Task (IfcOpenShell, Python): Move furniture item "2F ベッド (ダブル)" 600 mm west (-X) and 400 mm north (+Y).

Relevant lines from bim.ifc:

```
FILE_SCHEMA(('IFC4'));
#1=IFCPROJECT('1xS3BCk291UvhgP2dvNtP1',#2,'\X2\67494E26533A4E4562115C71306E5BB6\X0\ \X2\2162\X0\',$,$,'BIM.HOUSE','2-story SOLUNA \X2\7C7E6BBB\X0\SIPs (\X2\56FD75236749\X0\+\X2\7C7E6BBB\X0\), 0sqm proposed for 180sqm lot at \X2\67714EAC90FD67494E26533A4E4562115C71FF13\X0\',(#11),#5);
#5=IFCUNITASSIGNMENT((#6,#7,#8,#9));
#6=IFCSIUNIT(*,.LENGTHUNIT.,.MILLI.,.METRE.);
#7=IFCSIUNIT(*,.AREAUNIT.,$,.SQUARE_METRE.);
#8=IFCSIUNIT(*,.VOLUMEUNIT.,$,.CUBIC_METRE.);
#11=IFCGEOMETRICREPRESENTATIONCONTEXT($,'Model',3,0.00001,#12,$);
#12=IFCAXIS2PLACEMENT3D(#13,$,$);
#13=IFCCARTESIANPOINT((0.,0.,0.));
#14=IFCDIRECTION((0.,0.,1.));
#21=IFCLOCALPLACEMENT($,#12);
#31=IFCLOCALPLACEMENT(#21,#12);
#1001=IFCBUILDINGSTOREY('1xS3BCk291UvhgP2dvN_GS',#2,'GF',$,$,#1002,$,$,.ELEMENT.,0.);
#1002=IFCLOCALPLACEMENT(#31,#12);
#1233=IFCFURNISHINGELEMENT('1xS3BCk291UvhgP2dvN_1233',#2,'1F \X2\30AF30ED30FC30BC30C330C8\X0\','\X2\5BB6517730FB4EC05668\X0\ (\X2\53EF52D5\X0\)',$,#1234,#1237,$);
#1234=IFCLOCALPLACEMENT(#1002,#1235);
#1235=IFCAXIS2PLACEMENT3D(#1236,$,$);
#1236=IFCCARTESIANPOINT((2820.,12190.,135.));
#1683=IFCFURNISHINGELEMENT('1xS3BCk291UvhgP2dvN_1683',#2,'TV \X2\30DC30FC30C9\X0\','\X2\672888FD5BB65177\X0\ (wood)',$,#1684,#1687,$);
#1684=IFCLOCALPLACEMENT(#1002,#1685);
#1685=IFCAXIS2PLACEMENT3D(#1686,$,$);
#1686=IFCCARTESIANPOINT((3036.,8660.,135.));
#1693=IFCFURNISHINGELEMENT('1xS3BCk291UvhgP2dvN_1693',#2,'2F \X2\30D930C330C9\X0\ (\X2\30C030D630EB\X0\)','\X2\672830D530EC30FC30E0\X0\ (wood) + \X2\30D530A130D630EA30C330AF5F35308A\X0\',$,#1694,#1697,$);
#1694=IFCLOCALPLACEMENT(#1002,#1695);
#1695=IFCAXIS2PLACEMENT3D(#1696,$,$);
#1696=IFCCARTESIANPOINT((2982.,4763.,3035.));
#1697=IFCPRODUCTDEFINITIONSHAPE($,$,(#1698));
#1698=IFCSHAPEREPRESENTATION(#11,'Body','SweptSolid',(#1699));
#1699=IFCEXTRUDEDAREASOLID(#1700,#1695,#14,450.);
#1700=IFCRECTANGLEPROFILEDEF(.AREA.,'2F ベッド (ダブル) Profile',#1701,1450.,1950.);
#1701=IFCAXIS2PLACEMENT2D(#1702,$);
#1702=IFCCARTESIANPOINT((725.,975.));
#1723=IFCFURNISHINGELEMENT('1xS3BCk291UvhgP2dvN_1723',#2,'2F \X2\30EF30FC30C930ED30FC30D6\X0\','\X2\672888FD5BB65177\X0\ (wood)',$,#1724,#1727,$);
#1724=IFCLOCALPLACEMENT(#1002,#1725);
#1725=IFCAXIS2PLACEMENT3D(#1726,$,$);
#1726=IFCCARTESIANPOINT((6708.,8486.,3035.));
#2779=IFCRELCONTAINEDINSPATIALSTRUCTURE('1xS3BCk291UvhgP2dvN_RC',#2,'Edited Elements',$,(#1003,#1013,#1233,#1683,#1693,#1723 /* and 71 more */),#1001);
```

```python
import ifcopenshell
import ifcopenshell.api.geometry
import ifcopenshell.util.placement

model = ifcopenshell.open("bim.ifc")

item = model.by_guid("1xS3BCk291UvhgP2dvN_1693")
matrix = ifcopenshell.util.placement.get_local_placement(item.ObjectPlacement)
matrix[0, 3] -= 600.0
matrix[1, 3] += 400.0
ifcopenshell.api.geometry.edit_object_placement(model, product=item, matrix=matrix, is_si=False)

print(ifcopenshell.util.placement.get_local_placement(item.ObjectPlacement).round(3) + 0.0)

model.write("bim_updated.ifc")
```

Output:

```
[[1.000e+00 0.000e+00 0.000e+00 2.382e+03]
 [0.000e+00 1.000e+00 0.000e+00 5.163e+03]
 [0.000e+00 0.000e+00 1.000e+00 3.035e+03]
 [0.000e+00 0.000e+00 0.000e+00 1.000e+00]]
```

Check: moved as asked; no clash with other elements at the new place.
